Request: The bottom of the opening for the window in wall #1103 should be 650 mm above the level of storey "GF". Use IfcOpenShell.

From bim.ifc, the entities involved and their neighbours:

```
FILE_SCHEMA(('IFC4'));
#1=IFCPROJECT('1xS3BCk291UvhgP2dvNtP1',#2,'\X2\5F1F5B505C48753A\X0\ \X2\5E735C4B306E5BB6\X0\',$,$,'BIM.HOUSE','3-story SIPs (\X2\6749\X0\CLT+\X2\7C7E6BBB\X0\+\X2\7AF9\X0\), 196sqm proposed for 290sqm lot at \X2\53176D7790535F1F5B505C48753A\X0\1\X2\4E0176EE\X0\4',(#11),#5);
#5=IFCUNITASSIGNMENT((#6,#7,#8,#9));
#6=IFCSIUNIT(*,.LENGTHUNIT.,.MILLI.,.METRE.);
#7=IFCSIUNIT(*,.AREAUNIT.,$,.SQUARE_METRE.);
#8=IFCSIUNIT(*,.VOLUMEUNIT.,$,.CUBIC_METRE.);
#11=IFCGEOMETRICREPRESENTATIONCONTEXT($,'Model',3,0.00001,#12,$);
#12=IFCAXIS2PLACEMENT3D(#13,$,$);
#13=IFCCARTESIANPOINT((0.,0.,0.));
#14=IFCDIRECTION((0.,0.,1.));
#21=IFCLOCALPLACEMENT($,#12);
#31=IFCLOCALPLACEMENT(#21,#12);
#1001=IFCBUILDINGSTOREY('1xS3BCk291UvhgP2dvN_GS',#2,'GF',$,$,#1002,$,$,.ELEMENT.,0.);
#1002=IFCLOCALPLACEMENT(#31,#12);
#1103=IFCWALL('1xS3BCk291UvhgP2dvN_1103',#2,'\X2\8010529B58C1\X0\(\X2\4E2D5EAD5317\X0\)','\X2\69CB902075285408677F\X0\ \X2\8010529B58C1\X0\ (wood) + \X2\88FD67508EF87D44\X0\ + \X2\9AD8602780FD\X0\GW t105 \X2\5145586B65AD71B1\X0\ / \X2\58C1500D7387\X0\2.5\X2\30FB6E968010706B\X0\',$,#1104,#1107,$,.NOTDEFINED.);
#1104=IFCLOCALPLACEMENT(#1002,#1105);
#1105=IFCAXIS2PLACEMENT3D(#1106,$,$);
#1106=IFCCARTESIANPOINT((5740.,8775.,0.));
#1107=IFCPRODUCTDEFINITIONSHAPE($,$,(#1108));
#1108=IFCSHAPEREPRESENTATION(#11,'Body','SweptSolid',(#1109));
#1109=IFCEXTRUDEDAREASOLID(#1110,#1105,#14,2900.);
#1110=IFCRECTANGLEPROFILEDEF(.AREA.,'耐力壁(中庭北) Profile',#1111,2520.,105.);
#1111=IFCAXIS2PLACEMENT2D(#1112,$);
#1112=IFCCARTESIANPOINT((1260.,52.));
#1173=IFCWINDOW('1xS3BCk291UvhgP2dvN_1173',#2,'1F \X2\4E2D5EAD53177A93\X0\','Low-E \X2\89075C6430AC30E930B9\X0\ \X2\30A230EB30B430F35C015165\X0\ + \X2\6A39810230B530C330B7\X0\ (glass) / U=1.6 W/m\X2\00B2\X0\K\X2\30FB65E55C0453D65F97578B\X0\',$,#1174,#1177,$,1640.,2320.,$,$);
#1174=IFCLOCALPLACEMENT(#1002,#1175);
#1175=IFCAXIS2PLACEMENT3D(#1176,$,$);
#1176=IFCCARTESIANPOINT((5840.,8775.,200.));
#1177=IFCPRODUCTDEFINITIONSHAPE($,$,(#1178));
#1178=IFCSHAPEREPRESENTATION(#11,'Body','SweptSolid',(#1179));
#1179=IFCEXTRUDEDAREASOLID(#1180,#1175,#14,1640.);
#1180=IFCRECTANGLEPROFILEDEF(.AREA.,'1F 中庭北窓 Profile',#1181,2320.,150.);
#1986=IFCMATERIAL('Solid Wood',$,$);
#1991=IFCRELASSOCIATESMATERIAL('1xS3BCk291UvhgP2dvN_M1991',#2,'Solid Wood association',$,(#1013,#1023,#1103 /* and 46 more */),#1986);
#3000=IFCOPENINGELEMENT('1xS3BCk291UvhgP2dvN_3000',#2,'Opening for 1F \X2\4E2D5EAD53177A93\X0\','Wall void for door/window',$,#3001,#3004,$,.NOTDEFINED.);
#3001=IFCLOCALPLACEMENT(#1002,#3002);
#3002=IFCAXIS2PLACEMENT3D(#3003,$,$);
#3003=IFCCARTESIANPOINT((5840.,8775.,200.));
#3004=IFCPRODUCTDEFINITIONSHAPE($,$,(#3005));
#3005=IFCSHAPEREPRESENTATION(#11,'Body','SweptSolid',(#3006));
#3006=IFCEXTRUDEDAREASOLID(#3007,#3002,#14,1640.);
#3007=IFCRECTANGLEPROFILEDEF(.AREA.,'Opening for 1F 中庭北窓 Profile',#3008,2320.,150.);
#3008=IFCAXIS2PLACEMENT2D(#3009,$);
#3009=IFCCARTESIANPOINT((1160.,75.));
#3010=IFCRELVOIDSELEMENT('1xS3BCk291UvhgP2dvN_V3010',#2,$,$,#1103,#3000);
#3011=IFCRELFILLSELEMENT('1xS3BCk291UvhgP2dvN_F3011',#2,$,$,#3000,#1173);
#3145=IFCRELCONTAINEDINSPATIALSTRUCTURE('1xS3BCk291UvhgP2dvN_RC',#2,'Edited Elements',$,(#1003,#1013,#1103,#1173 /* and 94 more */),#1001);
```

```python
import numpy as np
import ifcopenshell
import ifcopenshell.api.geometry
import ifcopenshell.geom
import ifcopenshell.util.element
import ifcopenshell.util.placement
import ifcopenshell.util.shape
import ifcopenshell.util.unit

model = ifcopenshell.open("bim.ifc")
unit_scale = ifcopenshell.util.unit.calculate_unit_scale(model)

window = model.by_id(1173)
opening = window.FillsVoids[0].RelatingOpeningElement
storey = ifcopenshell.util.element.get_container(window, ifc_class="IfcBuildingStorey")
level = ifcopenshell.util.placement.get_local_placement(storey.ObjectPlacement)[2, 3]

# The opening's origin need not be at the sill, so measure its lowest point.
shape = ifcopenshell.geom.create_shape(ifcopenshell.geom.settings(), opening)
bottom = ifcopenshell.util.shape.get_shape_bottom_elevation(shape, shape.geometry) / unit_scale
dz = level + 650.0 - bottom

shift = np.array([0.0, 0.0, dz])
# The window is not placed relative to its opening, so move both.
for product in (opening, window):
    matrix = ifcopenshell.util.placement.get_local_placement(product.ObjectPlacement)
    matrix[:3, 3] += shift
    ifcopenshell.api.geometry.edit_object_placement(model, product=product, matrix=matrix, is_si=False)

print(f"moved by {dz * unit_scale:+.3f} m")

model.write("bim_v2.ifc")
```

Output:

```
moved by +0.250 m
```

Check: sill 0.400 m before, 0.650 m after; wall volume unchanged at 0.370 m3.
